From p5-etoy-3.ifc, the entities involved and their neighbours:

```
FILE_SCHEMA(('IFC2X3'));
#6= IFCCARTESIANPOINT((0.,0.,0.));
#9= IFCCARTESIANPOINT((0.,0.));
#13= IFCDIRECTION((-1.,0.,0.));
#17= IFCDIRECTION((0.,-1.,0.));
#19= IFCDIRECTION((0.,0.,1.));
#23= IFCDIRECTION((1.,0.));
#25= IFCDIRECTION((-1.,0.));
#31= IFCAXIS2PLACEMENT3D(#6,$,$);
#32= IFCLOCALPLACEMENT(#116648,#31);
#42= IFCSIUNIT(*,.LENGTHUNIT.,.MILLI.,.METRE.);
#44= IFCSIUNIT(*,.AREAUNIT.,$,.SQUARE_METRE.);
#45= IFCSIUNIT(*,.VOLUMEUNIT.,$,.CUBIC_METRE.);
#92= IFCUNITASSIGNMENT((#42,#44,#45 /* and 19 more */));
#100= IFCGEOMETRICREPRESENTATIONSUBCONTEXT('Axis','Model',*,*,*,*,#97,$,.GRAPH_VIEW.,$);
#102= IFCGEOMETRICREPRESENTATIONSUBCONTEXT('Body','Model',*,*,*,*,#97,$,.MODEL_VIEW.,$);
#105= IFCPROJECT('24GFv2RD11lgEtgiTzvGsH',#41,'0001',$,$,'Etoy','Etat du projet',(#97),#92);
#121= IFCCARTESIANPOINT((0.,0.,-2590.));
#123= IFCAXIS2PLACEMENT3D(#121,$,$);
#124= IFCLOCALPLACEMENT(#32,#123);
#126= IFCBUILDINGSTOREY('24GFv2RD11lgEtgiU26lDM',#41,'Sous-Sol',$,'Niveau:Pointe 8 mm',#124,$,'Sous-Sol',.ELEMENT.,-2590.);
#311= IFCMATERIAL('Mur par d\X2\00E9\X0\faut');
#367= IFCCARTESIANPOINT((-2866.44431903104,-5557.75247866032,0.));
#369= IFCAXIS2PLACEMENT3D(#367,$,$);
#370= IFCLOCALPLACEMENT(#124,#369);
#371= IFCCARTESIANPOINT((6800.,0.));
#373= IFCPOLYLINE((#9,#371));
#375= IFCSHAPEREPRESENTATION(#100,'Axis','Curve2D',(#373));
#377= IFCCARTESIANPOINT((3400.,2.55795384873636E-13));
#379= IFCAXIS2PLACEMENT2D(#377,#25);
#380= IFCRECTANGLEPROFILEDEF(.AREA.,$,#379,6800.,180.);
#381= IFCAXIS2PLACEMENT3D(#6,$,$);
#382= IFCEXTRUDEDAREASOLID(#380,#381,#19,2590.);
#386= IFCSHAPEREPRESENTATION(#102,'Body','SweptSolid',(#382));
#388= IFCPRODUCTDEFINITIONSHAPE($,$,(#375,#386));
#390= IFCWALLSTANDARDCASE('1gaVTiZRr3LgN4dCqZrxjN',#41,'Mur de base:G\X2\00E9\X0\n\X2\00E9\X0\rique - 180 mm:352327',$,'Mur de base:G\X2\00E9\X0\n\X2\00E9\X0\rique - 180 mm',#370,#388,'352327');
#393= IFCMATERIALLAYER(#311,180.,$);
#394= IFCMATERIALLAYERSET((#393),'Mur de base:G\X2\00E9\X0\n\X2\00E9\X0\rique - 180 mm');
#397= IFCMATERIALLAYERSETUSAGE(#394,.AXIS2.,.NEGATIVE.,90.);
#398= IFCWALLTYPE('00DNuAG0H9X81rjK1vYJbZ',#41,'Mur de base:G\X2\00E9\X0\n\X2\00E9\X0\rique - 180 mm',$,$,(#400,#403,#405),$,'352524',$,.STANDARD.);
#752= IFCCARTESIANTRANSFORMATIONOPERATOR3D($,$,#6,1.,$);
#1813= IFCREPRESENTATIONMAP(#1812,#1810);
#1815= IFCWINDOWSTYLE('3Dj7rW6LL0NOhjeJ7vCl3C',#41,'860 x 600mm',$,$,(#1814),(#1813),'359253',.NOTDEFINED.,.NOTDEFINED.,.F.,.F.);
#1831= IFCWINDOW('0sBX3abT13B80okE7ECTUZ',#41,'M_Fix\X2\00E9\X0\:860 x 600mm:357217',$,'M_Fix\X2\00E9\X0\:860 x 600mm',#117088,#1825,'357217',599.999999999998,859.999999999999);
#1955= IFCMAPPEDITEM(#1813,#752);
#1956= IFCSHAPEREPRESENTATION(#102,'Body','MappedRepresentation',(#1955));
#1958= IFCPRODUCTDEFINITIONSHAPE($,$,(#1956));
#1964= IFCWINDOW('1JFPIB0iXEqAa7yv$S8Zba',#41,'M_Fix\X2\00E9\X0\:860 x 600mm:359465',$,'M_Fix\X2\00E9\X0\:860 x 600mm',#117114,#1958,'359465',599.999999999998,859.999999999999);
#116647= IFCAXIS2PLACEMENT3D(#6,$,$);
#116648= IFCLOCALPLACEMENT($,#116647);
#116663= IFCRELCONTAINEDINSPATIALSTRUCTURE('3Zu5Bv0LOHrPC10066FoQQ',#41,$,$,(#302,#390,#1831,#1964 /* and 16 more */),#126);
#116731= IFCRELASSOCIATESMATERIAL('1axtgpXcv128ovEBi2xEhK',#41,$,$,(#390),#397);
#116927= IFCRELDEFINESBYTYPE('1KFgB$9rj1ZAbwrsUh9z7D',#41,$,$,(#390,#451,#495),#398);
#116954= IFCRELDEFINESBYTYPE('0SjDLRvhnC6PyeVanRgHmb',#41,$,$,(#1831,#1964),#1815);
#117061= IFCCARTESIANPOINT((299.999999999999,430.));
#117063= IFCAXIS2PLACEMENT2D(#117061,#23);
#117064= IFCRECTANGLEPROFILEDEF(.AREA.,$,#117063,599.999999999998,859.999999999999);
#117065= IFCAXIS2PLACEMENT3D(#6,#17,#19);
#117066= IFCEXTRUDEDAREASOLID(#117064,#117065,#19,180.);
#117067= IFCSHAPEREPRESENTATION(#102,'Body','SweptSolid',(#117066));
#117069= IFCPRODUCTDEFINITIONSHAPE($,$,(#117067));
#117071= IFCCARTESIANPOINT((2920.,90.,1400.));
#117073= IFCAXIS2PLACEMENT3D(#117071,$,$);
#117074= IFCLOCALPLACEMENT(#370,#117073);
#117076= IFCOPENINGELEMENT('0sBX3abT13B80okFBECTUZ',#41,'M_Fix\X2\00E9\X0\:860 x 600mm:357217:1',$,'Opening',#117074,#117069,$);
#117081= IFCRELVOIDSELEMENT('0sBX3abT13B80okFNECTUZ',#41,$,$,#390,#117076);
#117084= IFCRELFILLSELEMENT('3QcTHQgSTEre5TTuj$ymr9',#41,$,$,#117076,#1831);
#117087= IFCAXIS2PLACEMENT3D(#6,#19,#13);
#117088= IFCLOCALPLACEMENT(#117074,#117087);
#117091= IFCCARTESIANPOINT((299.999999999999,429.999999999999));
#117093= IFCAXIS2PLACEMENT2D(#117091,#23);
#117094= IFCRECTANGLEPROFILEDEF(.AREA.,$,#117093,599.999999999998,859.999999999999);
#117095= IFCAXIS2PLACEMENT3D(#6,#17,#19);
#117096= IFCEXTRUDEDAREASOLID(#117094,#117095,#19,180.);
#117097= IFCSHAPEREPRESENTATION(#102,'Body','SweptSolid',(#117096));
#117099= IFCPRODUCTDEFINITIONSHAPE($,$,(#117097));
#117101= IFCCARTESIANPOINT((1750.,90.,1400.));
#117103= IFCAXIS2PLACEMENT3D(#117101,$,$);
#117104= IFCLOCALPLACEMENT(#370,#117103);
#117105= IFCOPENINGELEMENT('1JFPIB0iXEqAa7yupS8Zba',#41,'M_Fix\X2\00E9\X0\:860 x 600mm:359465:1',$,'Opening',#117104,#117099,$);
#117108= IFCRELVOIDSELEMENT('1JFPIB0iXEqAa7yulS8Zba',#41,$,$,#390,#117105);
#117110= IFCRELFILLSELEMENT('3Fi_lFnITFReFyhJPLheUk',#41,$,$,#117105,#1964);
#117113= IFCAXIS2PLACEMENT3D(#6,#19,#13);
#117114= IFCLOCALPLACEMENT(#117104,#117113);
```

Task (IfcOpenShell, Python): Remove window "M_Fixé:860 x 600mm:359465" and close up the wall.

```python
import ifcopenshell
import ifcopenshell.api.feature
import ifcopenshell.api.root
import ifcopenshell.geom
import ifcopenshell.util.shape

model = ifcopenshell.open("p5-etoy-3.ifc")
settings = ifcopenshell.geom.settings()


def volume(element):
    """Net volume in cubic metres, openings subtracted."""
    shape = ifcopenshell.geom.create_shape(settings, element)
    return ifcopenshell.util.shape.get_volume(shape.geometry)


window = model.by_guid("1JFPIB0iXEqAa7yv$S8Zba")
opening = window.FillsVoids[0].RelatingOpeningElement
wall = opening.VoidsElements[0].RelatingBuildingElement
before = volume(wall)

ifcopenshell.api.root.remove_product(model, product=window)
ifcopenshell.api.feature.remove_feature(model, feature=opening)

after = volume(wall)

print(f"wall volume {before:.3f} -> {after:.3f} m3")

model.write("p5-etoy-3-out.ifc")
```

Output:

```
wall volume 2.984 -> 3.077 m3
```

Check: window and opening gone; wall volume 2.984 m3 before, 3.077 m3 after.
